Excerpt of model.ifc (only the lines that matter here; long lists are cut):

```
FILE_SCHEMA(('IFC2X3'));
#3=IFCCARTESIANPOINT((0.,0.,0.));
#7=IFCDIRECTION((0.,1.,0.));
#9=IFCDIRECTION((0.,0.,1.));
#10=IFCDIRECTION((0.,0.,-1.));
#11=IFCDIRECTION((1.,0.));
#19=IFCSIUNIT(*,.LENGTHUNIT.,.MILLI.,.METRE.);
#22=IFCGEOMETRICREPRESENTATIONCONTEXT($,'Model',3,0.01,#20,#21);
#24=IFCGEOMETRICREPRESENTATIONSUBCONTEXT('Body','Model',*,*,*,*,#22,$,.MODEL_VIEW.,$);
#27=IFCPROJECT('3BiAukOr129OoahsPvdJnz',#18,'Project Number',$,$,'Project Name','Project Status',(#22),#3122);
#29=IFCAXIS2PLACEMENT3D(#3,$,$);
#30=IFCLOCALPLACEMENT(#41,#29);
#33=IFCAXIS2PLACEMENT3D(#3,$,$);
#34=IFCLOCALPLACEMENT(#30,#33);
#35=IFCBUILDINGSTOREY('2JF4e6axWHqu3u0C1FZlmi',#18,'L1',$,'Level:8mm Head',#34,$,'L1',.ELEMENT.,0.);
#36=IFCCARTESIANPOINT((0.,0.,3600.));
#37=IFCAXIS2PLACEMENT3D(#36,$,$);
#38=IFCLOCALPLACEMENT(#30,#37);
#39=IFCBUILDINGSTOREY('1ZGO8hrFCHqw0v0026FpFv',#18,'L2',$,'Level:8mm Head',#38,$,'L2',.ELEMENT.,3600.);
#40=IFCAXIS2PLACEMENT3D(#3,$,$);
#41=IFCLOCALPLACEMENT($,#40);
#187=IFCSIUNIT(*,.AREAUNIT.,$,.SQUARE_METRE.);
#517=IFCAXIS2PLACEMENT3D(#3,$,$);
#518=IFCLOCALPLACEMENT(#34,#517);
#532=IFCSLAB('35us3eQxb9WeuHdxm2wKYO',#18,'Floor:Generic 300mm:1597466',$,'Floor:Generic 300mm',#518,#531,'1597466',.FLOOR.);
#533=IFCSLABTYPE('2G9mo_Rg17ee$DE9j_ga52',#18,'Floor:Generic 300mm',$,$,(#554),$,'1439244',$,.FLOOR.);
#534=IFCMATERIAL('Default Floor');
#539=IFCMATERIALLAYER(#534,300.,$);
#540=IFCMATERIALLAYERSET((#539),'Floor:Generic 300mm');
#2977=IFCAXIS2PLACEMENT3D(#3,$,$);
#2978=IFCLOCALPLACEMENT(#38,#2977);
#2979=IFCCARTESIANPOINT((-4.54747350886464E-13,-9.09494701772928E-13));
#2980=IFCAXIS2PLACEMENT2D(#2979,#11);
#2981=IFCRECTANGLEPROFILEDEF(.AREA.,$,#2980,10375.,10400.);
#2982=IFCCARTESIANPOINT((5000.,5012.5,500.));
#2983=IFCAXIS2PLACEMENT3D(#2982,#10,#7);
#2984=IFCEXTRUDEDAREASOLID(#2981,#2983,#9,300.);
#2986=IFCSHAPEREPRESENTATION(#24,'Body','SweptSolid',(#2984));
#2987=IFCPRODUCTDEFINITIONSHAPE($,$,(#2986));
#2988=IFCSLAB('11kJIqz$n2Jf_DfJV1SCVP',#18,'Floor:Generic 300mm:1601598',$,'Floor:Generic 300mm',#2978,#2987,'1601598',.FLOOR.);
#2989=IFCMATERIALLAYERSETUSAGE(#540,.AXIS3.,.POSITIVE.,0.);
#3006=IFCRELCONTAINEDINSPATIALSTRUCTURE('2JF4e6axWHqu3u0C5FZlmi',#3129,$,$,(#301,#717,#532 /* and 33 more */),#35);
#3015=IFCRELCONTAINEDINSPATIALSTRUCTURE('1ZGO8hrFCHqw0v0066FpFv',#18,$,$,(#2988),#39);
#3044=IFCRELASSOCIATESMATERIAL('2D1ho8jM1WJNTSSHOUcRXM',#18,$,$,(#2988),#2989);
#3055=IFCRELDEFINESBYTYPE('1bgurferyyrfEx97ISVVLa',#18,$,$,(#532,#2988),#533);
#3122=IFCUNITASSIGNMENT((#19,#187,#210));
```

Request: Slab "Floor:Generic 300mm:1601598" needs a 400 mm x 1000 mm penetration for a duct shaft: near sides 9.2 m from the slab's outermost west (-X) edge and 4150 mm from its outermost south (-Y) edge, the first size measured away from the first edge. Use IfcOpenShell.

```python
import numpy as np
import ifcopenshell
import ifcopenshell.api.feature
import ifcopenshell.api.geometry
import ifcopenshell.api.root
import ifcopenshell.geom
import ifcopenshell.util.placement
import ifcopenshell.util.representation
import ifcopenshell.util.shape
import ifcopenshell.util.unit

model = ifcopenshell.open("model.ifc")
unit_scale = ifcopenshell.util.unit.calculate_unit_scale(model)
settings = ifcopenshell.geom.settings()


def volume(element):
    """Net volume in cubic metres, openings subtracted."""
    shape = ifcopenshell.geom.create_shape(settings, element)
    return ifcopenshell.util.shape.get_volume(shape.geometry)


slab = model.by_guid("11kJIqz$n2Jf_DfJV1SCVP")
before = volume(slab)

# Extent in the slab's own axes, in metres. The edges named are its -X and -Y sides.
slab_shape = ifcopenshell.geom.create_shape(settings, slab)
vertices = ifcopenshell.util.shape.get_vertices(slab_shape.geometry)
x_min, y_min, bottom = vertices.min(axis=0)
top = vertices[:, 2].max()

opening = ifcopenshell.api.root.create_entity(model, ifc_class="IfcOpeningElement", name="Duct shaft opening")
context = ifcopenshell.util.representation.get_context(model, "Model", "Body", "MODEL_VIEW")
width, depth = 0.4, 1
outline = [(0.0, 0.0), (width, 0.0), (width, depth), (0.0, depth), (0.0, 0.0)]
# Overshoot both faces by 50 mm so the cut is clean.
shape = ifcopenshell.api.geometry.add_slab_representation(
    model, context=context, depth=top - bottom + 0.1, polyline=outline
)
ifcopenshell.api.geometry.assign_representation(model, product=opening, representation=shape)

matrix = ifcopenshell.util.placement.get_local_placement(slab.ObjectPlacement)
matrix[:, 3] = matrix @ np.append(np.array([x_min + 9.2, y_min + 4.15, bottom - 0.05]) / unit_scale, 1.0)
ifcopenshell.api.geometry.edit_object_placement(model, product=opening, matrix=matrix, is_si=False)
ifcopenshell.api.feature.add_feature(model, feature=opening, element=slab)

after = volume(slab)

print(f"slab volume {before:.3f} -> {after:.3f} m3")

model.write("model_v2.ifc")
```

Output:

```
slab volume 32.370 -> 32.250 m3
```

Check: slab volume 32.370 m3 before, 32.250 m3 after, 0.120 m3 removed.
